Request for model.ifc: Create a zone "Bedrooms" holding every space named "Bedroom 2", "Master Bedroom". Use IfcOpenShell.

First a look at what the model holds.

```python
import ifcopenshell

model = ifcopenshell.open("model.ifc")
print(model.schema)
seen = {}
for space in model.by_type("IfcSpace"):
    seen[space.LongName] = seen.get(space.LongName, 0) + 1
for name, count in sorted(seen.items(), key=str):
    print(count, "x", name)
print("zones:", [z.Name for z in model.by_type("IfcZone")][:20])
```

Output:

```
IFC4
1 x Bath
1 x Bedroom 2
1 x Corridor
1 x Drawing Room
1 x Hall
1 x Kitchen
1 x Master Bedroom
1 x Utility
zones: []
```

```python
import ifcopenshell
import ifcopenshell.api.group
import ifcopenshell.api.root

model = ifcopenshell.open("model.ifc")

names = {"Bedroom 2", "Master Bedroom"}
spaces = [s for s in model.by_type("IfcSpace") if s.LongName in names]

zone = ifcopenshell.api.root.create_entity(model, ifc_class="IfcZone", name="Bedrooms")
ifcopenshell.api.group.assign_group(model, products=spaces, group=zone)
print(len(spaces), "spaces in", zone.Name)

model.write("model-out.ifc")
```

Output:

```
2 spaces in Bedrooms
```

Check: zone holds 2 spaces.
